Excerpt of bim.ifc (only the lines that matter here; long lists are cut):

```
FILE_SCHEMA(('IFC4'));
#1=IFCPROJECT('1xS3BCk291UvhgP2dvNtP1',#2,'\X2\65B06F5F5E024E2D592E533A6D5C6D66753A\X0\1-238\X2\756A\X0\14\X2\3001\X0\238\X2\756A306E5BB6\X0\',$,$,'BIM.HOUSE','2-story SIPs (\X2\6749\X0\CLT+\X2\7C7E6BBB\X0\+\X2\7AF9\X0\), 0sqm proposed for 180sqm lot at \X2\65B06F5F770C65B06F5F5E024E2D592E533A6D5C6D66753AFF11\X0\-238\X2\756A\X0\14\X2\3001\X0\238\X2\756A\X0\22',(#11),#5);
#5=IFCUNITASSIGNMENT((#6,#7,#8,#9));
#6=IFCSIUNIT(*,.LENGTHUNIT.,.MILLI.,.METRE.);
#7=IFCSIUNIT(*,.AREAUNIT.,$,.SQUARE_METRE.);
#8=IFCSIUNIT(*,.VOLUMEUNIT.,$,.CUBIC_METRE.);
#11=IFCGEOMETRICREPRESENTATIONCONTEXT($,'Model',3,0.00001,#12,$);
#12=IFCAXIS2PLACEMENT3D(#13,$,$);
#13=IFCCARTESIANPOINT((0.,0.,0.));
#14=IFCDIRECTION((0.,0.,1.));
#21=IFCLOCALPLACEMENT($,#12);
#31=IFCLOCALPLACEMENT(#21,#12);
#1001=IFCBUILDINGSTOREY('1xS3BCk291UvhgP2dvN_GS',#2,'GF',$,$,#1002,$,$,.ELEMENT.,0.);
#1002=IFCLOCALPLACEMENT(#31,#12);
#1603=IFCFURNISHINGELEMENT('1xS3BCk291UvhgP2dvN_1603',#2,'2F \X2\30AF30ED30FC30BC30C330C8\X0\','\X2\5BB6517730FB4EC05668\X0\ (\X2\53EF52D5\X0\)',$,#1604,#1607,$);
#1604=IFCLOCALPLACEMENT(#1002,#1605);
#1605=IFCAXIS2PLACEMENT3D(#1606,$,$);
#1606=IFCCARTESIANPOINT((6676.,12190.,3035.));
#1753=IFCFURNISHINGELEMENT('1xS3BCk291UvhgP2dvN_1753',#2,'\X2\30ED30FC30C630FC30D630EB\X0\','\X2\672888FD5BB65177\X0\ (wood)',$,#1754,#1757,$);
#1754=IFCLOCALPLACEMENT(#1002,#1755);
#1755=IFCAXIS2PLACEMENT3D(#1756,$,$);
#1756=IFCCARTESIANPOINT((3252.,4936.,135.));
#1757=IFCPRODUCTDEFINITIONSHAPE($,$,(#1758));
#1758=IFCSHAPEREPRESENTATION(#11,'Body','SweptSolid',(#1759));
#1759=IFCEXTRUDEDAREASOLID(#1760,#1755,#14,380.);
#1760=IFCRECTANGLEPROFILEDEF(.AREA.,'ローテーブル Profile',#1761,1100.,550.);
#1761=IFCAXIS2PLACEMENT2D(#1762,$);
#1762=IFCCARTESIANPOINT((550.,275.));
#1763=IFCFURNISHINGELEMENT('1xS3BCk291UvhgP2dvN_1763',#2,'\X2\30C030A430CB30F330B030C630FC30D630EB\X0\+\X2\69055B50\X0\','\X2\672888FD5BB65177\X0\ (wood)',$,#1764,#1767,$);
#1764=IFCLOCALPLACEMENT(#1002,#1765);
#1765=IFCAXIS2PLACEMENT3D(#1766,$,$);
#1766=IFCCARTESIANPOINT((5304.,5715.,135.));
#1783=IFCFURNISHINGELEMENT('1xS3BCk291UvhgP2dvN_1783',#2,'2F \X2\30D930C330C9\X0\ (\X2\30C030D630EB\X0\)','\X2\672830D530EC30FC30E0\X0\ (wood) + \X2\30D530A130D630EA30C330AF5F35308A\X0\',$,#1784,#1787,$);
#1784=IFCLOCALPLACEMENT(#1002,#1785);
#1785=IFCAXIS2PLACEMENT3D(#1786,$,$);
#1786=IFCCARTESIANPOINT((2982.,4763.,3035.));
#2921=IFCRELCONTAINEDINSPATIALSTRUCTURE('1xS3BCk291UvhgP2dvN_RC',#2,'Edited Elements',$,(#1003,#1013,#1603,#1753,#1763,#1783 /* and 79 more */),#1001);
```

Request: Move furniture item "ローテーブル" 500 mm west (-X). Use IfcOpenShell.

```python
import ifcopenshell
import ifcopenshell.api.geometry
import ifcopenshell.util.placement

model = ifcopenshell.open("bim.ifc")

item = model.by_guid("1xS3BCk291UvhgP2dvN_1753")
matrix = ifcopenshell.util.placement.get_local_placement(item.ObjectPlacement)
matrix[0, 3] -= 500.0
ifcopenshell.api.geometry.edit_object_placement(model, product=item, matrix=matrix, is_si=False)

print(ifcopenshell.util.placement.get_local_placement(item.ObjectPlacement).round(3) + 0.0)

model.write("bim-out.ifc")
```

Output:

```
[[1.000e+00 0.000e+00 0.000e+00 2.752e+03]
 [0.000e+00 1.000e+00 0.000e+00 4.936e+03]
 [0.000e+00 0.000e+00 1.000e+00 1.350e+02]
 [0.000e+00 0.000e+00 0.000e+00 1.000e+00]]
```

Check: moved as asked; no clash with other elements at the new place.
